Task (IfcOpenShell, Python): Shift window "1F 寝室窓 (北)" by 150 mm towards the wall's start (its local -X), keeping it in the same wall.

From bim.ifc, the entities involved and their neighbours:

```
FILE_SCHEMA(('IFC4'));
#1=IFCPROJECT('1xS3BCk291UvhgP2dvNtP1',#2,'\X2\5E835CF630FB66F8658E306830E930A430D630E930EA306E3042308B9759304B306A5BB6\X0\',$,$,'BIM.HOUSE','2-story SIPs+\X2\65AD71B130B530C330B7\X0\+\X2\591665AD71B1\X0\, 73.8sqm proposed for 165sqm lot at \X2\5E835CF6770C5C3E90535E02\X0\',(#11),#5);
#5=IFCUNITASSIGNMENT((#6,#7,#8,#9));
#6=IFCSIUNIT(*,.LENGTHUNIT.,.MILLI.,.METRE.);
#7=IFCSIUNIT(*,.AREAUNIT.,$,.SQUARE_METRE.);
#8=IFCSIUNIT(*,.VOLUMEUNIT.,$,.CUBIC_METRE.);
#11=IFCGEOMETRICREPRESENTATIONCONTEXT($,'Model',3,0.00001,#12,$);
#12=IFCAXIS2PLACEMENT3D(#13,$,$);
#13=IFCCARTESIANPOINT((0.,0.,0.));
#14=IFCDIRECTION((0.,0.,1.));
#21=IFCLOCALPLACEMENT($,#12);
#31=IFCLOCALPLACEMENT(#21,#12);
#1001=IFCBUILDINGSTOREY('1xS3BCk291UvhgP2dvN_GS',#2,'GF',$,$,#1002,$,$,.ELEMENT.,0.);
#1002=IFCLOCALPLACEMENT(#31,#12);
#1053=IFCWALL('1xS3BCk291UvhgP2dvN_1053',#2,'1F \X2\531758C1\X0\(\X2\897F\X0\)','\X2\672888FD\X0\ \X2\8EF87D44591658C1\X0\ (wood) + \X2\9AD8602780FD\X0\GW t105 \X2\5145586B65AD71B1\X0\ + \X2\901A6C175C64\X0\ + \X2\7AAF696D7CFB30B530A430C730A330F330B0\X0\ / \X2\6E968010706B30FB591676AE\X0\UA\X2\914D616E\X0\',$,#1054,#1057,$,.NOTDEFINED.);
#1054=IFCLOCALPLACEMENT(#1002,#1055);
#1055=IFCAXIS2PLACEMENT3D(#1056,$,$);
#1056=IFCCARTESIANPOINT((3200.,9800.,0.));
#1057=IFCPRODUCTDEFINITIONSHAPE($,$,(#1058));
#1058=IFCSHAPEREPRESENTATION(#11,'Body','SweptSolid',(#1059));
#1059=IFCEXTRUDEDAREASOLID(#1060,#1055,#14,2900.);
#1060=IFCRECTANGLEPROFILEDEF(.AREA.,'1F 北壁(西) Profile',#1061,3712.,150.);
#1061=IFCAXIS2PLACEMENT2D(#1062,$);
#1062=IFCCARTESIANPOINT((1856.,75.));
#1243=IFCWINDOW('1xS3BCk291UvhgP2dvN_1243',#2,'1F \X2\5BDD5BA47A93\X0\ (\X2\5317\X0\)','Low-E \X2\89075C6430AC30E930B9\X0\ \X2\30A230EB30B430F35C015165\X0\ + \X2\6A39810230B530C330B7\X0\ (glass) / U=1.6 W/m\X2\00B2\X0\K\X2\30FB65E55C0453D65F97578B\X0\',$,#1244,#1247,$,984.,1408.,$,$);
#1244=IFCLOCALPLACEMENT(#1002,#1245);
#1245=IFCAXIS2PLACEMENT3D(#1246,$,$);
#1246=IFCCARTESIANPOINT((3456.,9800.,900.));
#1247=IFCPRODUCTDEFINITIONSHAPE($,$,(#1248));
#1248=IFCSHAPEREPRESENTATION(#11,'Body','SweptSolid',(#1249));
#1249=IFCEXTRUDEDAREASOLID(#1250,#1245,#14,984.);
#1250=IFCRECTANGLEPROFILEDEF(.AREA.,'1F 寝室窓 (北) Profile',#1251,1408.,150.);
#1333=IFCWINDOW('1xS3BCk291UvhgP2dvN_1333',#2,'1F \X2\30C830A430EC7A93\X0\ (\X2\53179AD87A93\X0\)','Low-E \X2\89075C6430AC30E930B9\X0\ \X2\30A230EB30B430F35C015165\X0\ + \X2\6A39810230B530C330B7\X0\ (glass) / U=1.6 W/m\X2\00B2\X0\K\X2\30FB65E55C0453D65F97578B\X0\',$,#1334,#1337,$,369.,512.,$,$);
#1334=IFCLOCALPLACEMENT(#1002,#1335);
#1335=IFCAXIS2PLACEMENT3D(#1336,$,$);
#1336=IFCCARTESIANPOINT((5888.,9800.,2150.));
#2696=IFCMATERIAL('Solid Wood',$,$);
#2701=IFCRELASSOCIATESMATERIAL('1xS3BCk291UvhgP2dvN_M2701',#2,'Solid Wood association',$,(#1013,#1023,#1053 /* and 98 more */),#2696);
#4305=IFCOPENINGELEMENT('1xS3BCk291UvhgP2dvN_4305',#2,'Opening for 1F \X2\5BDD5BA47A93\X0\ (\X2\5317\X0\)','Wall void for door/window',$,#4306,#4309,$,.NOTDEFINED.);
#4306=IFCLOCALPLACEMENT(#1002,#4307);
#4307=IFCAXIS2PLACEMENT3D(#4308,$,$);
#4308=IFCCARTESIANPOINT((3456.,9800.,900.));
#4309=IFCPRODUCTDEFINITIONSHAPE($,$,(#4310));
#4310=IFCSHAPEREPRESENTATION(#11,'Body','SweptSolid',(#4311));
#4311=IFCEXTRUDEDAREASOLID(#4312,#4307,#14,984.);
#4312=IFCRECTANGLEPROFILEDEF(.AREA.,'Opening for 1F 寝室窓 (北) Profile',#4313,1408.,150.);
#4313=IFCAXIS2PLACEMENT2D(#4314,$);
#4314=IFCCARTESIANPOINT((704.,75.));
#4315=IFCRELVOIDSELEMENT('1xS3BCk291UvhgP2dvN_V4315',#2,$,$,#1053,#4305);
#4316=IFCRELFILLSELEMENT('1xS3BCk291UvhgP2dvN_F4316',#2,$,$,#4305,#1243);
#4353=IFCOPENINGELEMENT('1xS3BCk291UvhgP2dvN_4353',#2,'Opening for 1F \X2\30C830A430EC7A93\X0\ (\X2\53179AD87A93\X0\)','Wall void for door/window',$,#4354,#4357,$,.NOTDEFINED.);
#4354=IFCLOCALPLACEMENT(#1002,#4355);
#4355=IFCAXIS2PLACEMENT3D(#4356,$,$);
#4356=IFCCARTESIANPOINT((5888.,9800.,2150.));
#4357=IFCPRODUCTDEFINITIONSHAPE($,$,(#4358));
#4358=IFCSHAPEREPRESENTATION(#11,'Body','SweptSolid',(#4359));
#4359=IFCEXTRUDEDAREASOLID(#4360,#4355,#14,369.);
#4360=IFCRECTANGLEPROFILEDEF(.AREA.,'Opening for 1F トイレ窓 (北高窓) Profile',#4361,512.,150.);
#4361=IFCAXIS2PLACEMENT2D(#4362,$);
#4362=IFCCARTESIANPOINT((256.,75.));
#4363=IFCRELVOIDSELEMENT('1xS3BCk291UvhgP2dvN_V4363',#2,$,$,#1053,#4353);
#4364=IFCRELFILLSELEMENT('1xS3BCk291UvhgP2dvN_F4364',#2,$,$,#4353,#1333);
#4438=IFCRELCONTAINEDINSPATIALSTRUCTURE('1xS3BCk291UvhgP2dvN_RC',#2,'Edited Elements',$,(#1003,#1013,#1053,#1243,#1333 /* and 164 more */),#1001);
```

```python
import ifcopenshell
import ifcopenshell.api.geometry
import ifcopenshell.util.placement
import ifcopenshell.util.unit

model = ifcopenshell.open("bim.ifc")
unit_scale = ifcopenshell.util.unit.calculate_unit_scale(model)

window = model.by_guid("1xS3BCk291UvhgP2dvN_1243")
opening = window.FillsVoids[0].RelatingOpeningElement
wall = opening.VoidsElements[0].RelatingBuildingElement

wall_matrix = ifcopenshell.util.placement.get_local_placement(wall.ObjectPlacement)
shift = wall_matrix[:3, 0] * -0.15 / unit_scale
before = ifcopenshell.util.placement.get_local_placement(window.ObjectPlacement)[:3, 3].copy()

# The window is not placed relative to its opening, so move both.
for product in (opening, window):
    matrix = ifcopenshell.util.placement.get_local_placement(product.ObjectPlacement)
    matrix[:3, 3] += shift
    ifcopenshell.api.geometry.edit_object_placement(model, product=product, matrix=matrix, is_si=False)

after = ifcopenshell.util.placement.get_local_placement(window.ObjectPlacement)[:3, 3]
print("window moved by", (after - before).round(3) + 0.0)

model.write("bim_updated.ifc")
```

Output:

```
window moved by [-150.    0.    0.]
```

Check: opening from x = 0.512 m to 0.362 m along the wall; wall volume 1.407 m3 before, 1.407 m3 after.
